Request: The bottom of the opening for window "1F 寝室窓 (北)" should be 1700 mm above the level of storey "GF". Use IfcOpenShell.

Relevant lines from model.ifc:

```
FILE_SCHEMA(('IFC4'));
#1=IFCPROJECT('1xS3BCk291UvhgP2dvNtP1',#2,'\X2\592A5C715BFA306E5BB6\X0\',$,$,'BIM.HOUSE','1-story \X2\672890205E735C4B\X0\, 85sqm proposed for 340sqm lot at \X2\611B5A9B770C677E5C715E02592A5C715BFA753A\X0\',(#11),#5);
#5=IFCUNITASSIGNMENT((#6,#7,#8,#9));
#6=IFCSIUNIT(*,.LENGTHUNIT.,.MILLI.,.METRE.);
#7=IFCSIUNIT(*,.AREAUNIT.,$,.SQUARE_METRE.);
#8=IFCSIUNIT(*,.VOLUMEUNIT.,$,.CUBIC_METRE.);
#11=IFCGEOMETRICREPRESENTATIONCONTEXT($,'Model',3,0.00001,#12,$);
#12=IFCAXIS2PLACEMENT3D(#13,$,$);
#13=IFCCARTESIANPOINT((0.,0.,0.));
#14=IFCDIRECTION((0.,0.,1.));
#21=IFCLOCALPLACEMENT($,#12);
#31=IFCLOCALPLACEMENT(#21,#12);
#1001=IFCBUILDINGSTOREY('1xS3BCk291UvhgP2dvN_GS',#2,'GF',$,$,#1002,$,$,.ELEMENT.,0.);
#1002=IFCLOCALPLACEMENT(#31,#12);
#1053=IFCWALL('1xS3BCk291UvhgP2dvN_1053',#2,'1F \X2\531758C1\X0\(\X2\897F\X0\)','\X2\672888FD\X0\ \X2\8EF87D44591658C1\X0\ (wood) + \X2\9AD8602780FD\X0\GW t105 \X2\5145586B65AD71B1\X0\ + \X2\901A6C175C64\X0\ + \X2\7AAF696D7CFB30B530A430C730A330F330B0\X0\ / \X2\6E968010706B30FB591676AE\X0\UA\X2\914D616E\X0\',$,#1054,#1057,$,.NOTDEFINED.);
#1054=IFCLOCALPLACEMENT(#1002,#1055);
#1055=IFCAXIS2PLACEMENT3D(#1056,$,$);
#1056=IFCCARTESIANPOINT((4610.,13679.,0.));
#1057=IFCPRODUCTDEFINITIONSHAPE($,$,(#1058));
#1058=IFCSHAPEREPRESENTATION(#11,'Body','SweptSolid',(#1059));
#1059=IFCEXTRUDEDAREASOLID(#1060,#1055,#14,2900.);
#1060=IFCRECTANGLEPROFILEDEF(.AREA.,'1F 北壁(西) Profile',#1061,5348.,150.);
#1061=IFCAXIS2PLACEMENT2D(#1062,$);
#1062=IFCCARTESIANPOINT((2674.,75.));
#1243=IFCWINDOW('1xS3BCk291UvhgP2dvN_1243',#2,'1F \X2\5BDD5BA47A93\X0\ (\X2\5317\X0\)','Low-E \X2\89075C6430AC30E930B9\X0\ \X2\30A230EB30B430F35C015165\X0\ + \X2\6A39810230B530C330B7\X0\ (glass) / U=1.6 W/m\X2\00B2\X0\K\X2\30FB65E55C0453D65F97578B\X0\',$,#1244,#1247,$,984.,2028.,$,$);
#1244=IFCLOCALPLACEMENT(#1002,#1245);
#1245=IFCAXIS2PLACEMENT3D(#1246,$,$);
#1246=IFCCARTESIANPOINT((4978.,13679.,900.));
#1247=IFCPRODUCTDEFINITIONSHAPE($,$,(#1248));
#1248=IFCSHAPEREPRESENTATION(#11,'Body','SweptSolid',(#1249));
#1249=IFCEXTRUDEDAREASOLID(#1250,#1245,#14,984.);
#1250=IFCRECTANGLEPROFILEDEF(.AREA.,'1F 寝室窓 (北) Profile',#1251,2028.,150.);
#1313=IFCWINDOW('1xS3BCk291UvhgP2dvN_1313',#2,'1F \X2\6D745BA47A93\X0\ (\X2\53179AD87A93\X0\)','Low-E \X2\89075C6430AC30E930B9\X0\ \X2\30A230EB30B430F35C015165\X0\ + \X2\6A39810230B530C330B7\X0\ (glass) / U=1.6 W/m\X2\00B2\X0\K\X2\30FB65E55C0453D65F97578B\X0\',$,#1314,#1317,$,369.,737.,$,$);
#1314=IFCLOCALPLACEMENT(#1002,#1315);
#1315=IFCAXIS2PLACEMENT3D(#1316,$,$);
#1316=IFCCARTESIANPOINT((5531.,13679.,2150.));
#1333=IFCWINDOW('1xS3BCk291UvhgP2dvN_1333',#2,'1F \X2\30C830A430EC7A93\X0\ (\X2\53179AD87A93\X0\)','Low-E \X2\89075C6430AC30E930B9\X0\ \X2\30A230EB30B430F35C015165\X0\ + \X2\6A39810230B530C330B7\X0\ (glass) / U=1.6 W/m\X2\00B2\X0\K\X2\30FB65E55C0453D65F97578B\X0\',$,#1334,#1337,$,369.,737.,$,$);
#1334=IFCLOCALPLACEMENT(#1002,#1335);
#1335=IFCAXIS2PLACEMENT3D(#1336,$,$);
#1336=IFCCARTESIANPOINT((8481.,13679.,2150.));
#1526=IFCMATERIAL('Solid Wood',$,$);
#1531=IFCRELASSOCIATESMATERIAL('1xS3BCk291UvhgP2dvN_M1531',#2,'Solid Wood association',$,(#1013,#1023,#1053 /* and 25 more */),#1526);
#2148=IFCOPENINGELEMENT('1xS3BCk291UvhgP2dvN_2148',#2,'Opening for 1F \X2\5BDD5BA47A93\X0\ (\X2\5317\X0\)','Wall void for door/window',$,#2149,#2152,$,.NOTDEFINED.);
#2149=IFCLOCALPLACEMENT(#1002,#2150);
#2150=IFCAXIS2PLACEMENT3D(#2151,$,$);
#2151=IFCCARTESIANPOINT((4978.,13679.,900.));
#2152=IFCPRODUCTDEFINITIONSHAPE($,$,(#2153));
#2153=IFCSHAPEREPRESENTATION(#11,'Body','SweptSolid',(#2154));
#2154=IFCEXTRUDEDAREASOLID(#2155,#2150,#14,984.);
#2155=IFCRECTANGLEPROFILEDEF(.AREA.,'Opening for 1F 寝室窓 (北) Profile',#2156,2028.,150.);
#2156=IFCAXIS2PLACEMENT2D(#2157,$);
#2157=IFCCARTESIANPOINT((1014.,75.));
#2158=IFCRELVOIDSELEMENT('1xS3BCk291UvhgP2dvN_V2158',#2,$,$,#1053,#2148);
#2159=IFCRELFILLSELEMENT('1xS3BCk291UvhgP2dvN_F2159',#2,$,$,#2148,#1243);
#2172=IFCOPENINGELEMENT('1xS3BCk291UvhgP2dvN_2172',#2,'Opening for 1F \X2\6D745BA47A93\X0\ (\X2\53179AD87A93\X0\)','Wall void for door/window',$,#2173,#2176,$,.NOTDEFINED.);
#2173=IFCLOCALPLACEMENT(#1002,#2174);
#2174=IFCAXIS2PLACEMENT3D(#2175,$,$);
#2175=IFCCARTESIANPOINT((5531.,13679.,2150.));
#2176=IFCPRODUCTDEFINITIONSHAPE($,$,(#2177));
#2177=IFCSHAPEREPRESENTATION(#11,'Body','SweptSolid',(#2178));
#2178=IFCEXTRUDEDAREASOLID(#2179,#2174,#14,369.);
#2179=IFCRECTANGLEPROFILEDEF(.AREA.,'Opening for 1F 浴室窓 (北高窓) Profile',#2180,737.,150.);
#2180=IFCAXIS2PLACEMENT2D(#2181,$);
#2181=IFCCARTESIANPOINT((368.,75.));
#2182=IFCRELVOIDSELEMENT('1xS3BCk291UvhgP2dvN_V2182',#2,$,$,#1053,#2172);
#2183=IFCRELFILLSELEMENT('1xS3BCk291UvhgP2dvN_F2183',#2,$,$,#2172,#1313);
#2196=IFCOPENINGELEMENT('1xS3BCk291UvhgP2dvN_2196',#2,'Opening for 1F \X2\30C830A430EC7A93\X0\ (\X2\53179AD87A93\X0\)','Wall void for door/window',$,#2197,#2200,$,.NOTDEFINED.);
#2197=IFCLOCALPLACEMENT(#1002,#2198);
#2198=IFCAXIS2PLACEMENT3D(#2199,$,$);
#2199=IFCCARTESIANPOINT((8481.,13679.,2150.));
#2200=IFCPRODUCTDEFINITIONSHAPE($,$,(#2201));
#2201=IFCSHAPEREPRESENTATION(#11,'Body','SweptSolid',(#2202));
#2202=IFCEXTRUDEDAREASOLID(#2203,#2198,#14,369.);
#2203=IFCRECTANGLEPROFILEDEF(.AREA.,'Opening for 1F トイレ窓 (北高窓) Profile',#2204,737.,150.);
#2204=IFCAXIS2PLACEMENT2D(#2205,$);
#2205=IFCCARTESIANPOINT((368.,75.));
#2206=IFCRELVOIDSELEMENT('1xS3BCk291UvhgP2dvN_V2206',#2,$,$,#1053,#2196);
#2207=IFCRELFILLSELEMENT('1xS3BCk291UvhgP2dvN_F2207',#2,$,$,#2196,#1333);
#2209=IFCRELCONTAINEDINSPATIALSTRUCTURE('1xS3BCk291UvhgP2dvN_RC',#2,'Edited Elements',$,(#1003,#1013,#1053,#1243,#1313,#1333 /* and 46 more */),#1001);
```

```python
import numpy as np
import ifcopenshell
import ifcopenshell.api.geometry
import ifcopenshell.geom
import ifcopenshell.util.element
import ifcopenshell.util.placement
import ifcopenshell.util.shape
import ifcopenshell.util.unit

model = ifcopenshell.open("model.ifc")
unit_scale = ifcopenshell.util.unit.calculate_unit_scale(model)

window = model.by_id(1243)
opening = window.FillsVoids[0].RelatingOpeningElement
storey = ifcopenshell.util.element.get_container(window, ifc_class="IfcBuildingStorey")
level = ifcopenshell.util.placement.get_local_placement(storey.ObjectPlacement)[2, 3]

# The opening's origin need not be at the sill, so measure its lowest point.
shape = ifcopenshell.geom.create_shape(ifcopenshell.geom.settings(), opening)
bottom = ifcopenshell.util.shape.get_shape_bottom_elevation(shape, shape.geometry) / unit_scale
dz = level + 1.7 / unit_scale - bottom

shift = np.array([0.0, 0.0, dz])
# The window is not placed relative to its opening, so move both.
for product in (opening, window):
    matrix = ifcopenshell.util.placement.get_local_placement(product.ObjectPlacement)
    matrix[:3, 3] += shift
    ifcopenshell.api.geometry.edit_object_placement(model, product=product, matrix=matrix, is_si=False)

print(f"moved by {dz * unit_scale:+.3f} m")

model.write("model_v2.ifc")
```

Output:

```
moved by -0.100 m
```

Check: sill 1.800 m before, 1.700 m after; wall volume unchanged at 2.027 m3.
